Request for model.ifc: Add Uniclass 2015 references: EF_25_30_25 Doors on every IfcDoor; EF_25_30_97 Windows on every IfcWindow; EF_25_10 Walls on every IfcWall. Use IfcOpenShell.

First a look at what the model holds.

```python
import ifcopenshell

model = ifcopenshell.open("model.ifc")
print(model.schema)
print("classifications:", [c.Name for c in model.by_type("IfcClassification")])
for ifc_class in ("IfcDoor", "IfcRoof", "IfcStair", "IfcWall", "IfcWindow"):
    print(ifc_class, len(model.by_type(ifc_class)))
```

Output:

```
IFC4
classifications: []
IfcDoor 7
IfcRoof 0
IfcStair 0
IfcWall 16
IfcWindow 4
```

```python
import ifcopenshell
import ifcopenshell.api.classification

model = ifcopenshell.open("model.ifc")

system = ifcopenshell.api.classification.add_classification(model, classification="Uniclass 2015")

codes = {
    "IfcDoor": ("EF_25_30_25", "Doors"),
    "IfcWindow": ("EF_25_30_97", "Windows"),
    "IfcWall": ("EF_25_10", "Walls"),
}
for ifc_class, (code, name) in codes.items():
    products = model.by_type(ifc_class)
    ifcopenshell.api.classification.add_reference(
        model, products=products, classification=system, identification=code, name=name
    )
    print(code, len(products))

model.write("model_updated.ifc")
```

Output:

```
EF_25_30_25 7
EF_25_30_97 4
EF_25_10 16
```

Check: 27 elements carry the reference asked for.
